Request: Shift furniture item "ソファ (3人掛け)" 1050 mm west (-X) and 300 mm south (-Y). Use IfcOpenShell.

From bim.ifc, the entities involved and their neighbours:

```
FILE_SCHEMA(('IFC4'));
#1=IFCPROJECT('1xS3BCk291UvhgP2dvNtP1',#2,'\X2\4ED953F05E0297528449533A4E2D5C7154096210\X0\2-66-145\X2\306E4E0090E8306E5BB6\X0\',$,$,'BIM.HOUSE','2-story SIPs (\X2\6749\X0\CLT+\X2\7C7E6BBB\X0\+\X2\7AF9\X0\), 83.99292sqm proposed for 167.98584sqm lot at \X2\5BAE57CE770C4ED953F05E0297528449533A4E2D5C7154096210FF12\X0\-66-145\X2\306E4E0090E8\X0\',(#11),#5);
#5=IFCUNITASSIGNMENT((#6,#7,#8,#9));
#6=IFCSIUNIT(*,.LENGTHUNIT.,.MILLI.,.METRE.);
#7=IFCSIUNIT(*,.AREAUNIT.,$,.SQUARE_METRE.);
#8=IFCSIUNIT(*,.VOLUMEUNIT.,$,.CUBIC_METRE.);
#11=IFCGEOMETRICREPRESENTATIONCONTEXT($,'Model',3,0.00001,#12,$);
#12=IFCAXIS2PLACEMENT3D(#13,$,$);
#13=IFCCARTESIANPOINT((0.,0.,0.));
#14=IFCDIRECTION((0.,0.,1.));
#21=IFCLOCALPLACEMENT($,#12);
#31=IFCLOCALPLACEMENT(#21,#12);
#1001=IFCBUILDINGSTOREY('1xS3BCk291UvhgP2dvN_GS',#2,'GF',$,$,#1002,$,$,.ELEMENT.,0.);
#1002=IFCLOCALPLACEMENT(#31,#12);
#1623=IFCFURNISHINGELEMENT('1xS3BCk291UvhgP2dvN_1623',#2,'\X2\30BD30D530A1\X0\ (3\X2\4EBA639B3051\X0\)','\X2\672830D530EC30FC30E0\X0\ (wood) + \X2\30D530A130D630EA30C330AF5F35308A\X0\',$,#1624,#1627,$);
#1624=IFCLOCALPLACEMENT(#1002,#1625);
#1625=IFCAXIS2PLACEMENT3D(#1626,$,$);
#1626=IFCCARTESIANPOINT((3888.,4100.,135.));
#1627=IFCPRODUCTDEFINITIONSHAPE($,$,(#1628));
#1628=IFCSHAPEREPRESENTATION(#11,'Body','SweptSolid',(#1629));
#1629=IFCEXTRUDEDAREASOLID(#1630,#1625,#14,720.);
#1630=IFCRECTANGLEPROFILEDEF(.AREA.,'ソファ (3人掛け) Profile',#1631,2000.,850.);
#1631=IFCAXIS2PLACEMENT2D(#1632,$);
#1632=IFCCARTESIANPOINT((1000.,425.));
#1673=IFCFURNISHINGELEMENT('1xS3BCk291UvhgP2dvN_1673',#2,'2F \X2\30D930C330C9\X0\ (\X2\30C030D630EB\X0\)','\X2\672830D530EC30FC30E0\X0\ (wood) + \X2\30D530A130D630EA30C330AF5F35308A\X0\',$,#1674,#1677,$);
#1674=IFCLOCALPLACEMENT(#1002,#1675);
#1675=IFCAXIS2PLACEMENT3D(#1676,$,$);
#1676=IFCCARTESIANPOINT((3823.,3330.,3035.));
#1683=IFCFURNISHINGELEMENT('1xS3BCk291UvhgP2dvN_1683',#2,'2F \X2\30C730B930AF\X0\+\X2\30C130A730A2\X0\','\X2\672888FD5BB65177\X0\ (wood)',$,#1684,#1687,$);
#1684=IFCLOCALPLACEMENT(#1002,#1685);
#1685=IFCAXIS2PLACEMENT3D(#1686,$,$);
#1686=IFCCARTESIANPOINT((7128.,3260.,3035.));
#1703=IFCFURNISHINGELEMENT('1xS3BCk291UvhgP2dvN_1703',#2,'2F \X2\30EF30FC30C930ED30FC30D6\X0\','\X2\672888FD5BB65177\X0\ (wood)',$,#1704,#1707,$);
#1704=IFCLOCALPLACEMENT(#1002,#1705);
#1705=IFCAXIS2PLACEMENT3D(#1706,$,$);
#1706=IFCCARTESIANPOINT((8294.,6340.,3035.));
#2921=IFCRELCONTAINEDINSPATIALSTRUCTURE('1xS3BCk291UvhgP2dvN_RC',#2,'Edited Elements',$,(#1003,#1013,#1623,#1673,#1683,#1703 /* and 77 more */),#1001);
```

```python
import ifcopenshell
import ifcopenshell.api.geometry
import ifcopenshell.util.placement
import ifcopenshell.util.unit

model = ifcopenshell.open("bim.ifc")
unit_scale = ifcopenshell.util.unit.calculate_unit_scale(model)

item = model.by_guid("1xS3BCk291UvhgP2dvN_1623")
matrix = ifcopenshell.util.placement.get_local_placement(item.ObjectPlacement)
matrix[0, 3] -= 1.05 / unit_scale
matrix[1, 3] -= 0.3 / unit_scale
ifcopenshell.api.geometry.edit_object_placement(model, product=item, matrix=matrix, is_si=False)

print(ifcopenshell.util.placement.get_local_placement(item.ObjectPlacement).round(3) + 0.0)

model.write("bim_updated.ifc")
```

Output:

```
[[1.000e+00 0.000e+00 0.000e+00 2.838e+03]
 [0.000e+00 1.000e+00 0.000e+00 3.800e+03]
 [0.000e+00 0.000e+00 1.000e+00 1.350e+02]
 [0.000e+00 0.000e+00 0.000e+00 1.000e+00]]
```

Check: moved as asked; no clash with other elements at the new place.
